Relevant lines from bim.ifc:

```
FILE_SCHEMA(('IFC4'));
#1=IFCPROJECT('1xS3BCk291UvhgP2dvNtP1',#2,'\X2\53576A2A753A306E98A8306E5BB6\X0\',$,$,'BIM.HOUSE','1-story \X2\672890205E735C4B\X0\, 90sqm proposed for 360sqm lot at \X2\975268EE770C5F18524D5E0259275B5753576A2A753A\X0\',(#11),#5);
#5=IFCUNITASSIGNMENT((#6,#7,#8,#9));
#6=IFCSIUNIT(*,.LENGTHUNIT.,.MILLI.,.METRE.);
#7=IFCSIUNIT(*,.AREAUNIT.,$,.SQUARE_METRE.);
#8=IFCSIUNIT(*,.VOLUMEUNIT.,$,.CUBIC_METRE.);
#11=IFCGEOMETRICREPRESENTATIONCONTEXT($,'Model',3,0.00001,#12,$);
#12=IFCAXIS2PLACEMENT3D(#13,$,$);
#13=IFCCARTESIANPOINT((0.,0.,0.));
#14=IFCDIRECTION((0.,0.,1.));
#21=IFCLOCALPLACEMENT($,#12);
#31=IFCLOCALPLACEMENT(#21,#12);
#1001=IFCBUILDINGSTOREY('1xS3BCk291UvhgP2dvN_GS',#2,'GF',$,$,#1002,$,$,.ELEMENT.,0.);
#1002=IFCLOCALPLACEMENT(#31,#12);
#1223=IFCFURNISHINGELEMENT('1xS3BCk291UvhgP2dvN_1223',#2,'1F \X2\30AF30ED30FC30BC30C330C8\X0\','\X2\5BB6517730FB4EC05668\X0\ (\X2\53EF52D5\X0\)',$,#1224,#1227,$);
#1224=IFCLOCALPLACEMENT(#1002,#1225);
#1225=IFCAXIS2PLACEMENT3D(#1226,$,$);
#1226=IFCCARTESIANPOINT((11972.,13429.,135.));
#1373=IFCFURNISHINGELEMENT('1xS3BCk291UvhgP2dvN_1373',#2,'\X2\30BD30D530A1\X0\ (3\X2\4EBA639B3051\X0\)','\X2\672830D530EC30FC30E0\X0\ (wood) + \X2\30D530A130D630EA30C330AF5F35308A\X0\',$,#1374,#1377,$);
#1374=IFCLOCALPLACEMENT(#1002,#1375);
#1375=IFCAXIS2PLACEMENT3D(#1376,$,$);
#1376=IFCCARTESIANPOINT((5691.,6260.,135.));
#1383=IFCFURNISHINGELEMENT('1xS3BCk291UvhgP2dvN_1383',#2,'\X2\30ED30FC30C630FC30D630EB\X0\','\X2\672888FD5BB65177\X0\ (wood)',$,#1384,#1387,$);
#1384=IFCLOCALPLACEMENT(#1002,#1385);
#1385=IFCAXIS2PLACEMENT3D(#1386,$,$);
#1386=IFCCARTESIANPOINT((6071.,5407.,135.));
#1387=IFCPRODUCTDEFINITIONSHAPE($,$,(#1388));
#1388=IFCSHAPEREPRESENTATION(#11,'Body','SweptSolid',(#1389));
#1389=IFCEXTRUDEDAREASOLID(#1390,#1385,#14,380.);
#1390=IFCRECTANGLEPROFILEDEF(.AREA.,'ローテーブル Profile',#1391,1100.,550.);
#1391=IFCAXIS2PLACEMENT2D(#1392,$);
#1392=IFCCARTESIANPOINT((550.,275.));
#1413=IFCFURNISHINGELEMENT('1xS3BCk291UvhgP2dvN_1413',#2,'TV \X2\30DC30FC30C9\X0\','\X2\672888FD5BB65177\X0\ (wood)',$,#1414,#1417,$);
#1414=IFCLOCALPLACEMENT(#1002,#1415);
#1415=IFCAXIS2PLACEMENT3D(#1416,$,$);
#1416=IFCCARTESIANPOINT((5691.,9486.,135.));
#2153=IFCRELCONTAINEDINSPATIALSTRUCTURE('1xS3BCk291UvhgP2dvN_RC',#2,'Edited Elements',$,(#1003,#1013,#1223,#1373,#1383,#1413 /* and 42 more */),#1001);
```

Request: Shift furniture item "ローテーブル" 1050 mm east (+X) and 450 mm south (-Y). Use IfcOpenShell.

```python
import ifcopenshell
import ifcopenshell.api.geometry
import ifcopenshell.util.placement
import ifcopenshell.util.unit

model = ifcopenshell.open("bim.ifc")
unit_scale = ifcopenshell.util.unit.calculate_unit_scale(model)

item = model.by_guid("1xS3BCk291UvhgP2dvN_1383")
matrix = ifcopenshell.util.placement.get_local_placement(item.ObjectPlacement)
matrix[0, 3] += 1.05 / unit_scale
matrix[1, 3] -= 0.45 / unit_scale
ifcopenshell.api.geometry.edit_object_placement(model, product=item, matrix=matrix, is_si=False)

print(ifcopenshell.util.placement.get_local_placement(item.ObjectPlacement).round(3) + 0.0)

model.write("bim_rev.ifc")
```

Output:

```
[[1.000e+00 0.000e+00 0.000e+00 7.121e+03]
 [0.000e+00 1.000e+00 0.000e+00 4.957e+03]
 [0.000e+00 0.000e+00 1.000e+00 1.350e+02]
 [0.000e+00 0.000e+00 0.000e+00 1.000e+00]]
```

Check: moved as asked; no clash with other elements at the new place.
